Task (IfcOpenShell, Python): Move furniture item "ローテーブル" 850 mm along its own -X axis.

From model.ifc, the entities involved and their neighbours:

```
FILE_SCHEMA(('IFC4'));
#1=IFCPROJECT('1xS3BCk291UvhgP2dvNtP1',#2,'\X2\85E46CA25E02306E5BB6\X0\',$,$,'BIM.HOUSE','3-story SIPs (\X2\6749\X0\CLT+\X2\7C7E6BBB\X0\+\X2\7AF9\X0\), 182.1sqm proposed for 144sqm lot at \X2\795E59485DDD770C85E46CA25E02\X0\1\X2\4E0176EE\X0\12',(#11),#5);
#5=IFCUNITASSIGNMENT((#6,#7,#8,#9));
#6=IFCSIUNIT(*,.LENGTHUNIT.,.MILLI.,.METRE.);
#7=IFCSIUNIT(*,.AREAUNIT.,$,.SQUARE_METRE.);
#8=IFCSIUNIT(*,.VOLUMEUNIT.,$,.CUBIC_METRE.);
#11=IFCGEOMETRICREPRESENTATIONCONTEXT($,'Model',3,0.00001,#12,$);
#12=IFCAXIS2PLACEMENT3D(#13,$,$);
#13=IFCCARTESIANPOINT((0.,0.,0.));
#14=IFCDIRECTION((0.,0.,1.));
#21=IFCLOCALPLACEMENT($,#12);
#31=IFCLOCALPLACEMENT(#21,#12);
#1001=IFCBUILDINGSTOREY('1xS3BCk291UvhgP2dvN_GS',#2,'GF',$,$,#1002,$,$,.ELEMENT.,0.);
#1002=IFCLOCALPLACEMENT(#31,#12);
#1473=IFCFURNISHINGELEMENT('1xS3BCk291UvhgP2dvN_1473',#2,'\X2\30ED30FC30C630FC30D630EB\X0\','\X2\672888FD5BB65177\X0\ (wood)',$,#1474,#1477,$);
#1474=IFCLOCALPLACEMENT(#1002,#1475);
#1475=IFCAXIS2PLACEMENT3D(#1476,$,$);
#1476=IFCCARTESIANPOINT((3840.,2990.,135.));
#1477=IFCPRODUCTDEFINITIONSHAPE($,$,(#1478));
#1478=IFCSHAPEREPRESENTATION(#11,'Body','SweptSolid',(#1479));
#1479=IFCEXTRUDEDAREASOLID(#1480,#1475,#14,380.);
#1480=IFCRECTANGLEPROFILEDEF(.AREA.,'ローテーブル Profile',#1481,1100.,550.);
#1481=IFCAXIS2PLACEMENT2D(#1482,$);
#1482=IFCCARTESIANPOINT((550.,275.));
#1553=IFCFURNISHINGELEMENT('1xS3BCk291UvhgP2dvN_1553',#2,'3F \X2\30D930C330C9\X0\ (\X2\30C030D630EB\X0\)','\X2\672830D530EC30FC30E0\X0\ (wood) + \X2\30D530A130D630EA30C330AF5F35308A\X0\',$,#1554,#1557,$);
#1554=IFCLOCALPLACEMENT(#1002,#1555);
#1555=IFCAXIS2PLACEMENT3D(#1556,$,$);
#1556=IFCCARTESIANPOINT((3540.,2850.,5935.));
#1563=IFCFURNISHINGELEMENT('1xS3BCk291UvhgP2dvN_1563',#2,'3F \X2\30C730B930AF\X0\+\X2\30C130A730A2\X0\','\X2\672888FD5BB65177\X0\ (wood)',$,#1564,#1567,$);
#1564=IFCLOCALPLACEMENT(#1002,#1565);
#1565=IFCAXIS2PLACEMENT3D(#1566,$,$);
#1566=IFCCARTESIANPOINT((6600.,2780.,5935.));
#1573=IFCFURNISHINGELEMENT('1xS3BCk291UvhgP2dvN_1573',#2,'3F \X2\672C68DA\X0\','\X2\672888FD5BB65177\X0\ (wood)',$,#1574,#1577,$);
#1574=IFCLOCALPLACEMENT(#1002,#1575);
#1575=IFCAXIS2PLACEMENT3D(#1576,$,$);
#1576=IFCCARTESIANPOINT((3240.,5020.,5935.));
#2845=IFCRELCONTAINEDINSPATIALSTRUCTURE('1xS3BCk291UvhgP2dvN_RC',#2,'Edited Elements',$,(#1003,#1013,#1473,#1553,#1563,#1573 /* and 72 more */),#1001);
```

```python
import ifcopenshell
import ifcopenshell.api.geometry
import ifcopenshell.util.placement

model = ifcopenshell.open("model.ifc")

item = model.by_guid("1xS3BCk291UvhgP2dvN_1473")
matrix = ifcopenshell.util.placement.get_local_placement(item.ObjectPlacement)
matrix[:3, 3] -= matrix[:3, 0] * 850.0
ifcopenshell.api.geometry.edit_object_placement(model, product=item, matrix=matrix, is_si=False)

print(ifcopenshell.util.placement.get_local_placement(item.ObjectPlacement).round(3) + 0.0)

model.write("model-out.ifc")
```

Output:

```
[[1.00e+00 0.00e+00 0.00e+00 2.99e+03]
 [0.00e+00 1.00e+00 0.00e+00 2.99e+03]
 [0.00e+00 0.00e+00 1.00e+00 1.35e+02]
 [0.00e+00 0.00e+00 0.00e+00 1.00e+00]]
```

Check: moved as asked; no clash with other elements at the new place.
